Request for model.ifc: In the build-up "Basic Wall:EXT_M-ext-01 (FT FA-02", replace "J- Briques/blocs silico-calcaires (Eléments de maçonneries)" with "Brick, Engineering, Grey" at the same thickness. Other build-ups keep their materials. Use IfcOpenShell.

First a look at what the model holds.

```python
import ifcopenshell
import ifcopenshell.util.element

model = ifcopenshell.open("model.ifc")
print(model.schema)
for layer_set in model.by_type("IfcMaterialLayerSet"):
    if layer_set.LayerSetName == "Basic Wall:EXT_M-ext-01 (FT FA-02":
        for layer in layer_set.MaterialLayers:
            print(layer.id(), layer.Material and layer.Material.Name, layer.LayerThickness, sep=" | ")
        print(len(ifcopenshell.util.element.get_elements_by_material(model, layer_set)), "elements and types use it")
print(sorted(m.Name for m in model.by_type("IfcMaterial") if m.Name)[:60])
```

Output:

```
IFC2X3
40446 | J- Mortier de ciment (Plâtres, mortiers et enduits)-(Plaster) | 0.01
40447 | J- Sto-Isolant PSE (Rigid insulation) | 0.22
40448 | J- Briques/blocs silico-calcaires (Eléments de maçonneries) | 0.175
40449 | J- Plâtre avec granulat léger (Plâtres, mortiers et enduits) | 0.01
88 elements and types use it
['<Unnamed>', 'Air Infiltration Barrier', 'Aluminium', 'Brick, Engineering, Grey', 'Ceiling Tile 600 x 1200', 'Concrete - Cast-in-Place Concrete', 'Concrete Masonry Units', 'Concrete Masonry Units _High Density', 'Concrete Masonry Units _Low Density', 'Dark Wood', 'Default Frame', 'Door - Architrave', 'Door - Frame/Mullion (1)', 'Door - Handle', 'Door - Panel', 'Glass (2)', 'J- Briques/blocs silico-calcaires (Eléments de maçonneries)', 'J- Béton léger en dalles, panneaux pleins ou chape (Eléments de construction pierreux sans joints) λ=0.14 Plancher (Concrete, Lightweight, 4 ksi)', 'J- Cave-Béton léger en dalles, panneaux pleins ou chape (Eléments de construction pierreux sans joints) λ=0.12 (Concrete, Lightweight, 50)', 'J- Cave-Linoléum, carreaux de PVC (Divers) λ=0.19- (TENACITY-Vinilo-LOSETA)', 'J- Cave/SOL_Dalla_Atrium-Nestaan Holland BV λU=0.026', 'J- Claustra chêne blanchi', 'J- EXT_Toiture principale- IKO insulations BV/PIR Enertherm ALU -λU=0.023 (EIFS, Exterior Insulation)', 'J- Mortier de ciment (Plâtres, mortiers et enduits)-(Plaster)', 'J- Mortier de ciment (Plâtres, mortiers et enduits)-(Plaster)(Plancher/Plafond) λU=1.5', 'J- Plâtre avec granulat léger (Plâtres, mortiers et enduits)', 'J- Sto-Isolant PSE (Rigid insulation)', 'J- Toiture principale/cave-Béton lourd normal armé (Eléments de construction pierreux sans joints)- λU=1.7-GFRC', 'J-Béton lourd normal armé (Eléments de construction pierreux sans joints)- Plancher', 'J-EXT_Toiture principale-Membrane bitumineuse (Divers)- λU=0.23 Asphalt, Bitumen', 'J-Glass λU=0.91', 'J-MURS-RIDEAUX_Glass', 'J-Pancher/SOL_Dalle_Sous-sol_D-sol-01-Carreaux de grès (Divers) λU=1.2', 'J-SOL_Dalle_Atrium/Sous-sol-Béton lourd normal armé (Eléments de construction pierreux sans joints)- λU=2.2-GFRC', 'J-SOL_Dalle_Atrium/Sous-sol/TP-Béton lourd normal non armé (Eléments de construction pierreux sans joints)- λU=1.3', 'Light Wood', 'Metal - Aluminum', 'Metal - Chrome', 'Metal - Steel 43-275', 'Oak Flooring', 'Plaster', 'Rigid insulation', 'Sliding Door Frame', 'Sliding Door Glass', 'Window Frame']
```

```python
import ifcopenshell
import ifcopenshell.api.material

model = ifcopenshell.open("model.ifc")

layer_set = next(s for s in model.by_type("IfcMaterialLayerSet") if s.LayerSetName == "Basic Wall:EXT_M-ext-01 (FT FA-02")
layer = next(l for l in layer_set.MaterialLayers if l.Material and l.Material.Name == "J- Briques/blocs silico-calcaires (Eléments de maçonneries)")
material = next(m for m in model.by_type("IfcMaterial") if m.Name == "Brick, Engineering, Grey")

# Point this one layer at the other material; renaming the old one would change it everywhere.
ifcopenshell.api.material.edit_layer(model, layer=layer, attributes={}, material=material)

print([l.Material.Name if l.Material else None for l in layer_set.MaterialLayers])

model.write("model_edited.ifc")
```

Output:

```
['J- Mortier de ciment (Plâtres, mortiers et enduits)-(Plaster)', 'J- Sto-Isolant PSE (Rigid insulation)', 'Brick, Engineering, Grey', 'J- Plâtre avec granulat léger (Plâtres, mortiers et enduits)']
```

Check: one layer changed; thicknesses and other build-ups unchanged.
